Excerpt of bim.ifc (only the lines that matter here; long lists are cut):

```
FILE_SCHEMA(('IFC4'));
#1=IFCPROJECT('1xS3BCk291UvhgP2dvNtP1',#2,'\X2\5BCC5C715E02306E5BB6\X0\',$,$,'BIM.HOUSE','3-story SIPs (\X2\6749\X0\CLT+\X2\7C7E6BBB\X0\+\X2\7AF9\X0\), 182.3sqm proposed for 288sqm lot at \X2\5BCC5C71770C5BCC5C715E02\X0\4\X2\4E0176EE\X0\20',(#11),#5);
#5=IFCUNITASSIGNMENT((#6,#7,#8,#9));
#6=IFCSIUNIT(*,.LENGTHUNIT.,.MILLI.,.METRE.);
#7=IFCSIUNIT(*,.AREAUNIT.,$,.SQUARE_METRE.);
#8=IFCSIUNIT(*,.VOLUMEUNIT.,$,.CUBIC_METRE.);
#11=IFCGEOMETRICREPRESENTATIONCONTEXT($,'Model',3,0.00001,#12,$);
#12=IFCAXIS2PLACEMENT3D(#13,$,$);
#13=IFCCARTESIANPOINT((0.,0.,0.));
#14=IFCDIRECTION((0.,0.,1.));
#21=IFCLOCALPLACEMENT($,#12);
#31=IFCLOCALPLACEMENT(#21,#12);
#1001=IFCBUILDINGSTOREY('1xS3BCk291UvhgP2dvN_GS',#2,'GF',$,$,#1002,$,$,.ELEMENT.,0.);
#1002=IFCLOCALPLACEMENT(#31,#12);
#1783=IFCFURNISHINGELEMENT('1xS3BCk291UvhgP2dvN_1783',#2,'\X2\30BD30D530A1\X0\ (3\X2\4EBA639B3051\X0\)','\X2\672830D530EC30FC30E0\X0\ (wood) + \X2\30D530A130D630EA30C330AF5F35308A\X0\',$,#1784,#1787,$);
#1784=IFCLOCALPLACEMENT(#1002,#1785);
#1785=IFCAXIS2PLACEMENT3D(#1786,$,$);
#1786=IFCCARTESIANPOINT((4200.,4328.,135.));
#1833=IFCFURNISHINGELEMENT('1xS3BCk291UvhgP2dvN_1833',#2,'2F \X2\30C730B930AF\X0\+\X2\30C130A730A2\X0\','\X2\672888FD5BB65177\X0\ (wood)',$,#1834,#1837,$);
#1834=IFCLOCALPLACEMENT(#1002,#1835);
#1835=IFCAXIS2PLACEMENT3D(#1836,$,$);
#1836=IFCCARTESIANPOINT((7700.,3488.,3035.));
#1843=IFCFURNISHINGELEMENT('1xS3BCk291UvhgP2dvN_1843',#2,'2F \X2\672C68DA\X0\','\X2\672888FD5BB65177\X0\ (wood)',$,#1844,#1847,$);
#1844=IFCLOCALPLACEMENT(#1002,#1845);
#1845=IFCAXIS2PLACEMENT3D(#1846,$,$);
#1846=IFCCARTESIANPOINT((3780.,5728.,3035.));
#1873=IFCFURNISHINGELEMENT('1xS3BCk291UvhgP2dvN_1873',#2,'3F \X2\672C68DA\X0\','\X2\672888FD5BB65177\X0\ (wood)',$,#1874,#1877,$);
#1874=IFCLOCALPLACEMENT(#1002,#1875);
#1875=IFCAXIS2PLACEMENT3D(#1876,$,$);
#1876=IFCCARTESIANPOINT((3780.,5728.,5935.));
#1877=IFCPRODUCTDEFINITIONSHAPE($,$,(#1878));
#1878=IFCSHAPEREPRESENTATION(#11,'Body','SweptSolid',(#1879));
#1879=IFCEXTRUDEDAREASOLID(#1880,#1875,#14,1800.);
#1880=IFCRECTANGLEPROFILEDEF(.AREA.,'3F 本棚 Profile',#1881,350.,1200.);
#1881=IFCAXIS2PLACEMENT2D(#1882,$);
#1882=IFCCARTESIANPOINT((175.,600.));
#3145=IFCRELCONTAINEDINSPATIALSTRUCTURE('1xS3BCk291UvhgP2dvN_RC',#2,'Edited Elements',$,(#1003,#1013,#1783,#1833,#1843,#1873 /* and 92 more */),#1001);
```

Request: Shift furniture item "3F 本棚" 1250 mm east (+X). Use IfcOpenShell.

```python
import ifcopenshell
import ifcopenshell.api.geometry
import ifcopenshell.util.placement

model = ifcopenshell.open("bim.ifc")

item = model.by_guid("1xS3BCk291UvhgP2dvN_1873")
matrix = ifcopenshell.util.placement.get_local_placement(item.ObjectPlacement)
matrix[0, 3] += 1250.0
ifcopenshell.api.geometry.edit_object_placement(model, product=item, matrix=matrix, is_si=False)

print(ifcopenshell.util.placement.get_local_placement(item.ObjectPlacement).round(3) + 0.0)

model.write("bim-out.ifc")
```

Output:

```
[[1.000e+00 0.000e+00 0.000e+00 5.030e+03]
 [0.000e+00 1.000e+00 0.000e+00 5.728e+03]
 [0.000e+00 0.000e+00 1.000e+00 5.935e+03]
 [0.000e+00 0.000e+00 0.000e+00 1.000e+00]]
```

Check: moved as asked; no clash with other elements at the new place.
